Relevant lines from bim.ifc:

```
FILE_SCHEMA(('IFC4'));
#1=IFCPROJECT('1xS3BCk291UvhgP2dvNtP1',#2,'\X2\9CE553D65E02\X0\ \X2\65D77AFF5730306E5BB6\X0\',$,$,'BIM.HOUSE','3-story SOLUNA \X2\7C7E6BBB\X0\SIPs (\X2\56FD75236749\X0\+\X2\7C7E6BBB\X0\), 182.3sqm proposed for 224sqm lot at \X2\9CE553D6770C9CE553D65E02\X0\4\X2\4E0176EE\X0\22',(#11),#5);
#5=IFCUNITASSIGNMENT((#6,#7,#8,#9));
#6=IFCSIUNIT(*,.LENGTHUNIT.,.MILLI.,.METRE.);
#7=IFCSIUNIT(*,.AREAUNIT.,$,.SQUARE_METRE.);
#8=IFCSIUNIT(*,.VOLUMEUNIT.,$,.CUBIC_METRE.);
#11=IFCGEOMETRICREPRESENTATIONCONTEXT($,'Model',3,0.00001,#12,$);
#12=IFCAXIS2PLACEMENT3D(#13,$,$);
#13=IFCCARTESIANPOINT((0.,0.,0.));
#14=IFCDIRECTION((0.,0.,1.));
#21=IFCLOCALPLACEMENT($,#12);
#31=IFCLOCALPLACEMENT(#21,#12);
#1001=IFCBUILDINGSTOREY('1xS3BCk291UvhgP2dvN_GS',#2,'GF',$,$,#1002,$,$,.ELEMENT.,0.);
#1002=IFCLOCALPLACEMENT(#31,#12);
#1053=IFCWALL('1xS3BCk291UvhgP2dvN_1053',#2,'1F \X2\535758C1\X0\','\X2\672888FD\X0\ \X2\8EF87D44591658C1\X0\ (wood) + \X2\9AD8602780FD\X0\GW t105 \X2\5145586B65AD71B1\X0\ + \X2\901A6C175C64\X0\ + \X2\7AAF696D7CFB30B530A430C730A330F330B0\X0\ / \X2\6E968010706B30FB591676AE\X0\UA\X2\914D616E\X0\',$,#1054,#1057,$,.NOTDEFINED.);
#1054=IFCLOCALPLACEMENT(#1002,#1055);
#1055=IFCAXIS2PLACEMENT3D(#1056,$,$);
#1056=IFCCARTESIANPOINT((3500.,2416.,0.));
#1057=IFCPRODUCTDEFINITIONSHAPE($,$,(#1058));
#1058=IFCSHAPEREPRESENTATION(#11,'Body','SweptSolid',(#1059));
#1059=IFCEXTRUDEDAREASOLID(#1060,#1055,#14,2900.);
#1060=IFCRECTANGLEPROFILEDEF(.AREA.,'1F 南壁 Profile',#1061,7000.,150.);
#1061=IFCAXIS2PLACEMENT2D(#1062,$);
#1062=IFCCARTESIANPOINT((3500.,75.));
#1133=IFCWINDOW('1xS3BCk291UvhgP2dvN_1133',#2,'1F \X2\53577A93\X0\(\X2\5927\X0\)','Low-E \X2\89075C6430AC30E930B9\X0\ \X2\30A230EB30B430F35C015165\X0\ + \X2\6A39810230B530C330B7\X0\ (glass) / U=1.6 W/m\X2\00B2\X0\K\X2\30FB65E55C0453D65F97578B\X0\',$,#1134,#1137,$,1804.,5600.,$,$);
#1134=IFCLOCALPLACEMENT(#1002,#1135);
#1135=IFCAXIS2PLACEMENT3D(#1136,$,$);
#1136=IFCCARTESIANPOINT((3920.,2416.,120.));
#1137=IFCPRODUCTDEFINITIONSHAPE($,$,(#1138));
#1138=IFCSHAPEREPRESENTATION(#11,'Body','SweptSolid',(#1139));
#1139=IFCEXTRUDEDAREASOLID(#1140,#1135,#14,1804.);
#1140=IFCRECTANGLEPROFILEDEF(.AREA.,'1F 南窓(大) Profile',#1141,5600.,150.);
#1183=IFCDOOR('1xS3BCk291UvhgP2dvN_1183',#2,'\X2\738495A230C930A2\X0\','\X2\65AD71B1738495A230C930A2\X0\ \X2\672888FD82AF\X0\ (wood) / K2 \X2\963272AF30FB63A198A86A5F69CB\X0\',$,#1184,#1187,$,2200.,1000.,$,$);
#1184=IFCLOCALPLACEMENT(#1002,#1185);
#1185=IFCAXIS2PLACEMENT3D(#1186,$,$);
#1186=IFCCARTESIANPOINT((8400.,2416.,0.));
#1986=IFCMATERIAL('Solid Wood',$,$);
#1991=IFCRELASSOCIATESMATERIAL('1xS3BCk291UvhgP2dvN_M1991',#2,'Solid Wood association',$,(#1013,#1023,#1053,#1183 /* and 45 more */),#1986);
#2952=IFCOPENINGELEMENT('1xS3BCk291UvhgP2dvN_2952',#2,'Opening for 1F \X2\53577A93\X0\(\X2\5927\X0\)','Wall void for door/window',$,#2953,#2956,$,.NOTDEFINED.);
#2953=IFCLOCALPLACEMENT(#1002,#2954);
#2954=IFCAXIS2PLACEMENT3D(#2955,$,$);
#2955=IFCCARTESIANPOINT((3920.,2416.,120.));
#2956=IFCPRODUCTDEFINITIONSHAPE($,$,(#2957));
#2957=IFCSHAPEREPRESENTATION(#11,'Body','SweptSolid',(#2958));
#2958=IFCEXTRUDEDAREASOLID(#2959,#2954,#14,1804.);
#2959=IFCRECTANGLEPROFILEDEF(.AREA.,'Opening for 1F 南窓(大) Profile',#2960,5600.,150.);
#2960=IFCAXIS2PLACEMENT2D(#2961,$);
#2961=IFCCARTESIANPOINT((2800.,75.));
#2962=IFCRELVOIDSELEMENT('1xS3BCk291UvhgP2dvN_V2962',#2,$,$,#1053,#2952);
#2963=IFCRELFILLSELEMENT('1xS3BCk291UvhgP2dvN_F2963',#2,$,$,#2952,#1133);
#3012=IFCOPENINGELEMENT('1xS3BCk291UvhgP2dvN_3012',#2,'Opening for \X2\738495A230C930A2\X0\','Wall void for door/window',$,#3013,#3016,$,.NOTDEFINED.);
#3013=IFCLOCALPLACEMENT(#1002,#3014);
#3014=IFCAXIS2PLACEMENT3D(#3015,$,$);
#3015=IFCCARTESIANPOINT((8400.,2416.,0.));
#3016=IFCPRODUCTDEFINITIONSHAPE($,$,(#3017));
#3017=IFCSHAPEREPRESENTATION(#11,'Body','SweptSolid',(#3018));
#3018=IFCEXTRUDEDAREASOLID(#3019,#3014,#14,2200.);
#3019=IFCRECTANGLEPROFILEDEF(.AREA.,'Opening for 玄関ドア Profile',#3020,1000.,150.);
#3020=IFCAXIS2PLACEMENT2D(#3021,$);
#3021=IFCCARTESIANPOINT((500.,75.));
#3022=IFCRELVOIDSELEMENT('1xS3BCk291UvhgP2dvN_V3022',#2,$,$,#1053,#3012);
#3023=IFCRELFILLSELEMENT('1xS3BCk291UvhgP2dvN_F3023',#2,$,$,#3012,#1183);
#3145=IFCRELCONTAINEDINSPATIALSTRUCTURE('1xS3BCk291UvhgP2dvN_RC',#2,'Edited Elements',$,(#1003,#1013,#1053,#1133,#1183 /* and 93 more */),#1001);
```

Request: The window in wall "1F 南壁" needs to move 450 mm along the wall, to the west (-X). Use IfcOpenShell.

```python
import ifcopenshell
import ifcopenshell.api.geometry
import ifcopenshell.util.placement

model = ifcopenshell.open("bim.ifc")

window = model.by_guid("1xS3BCk291UvhgP2dvN_1133")
opening = window.FillsVoids[0].RelatingOpeningElement
wall = opening.VoidsElements[0].RelatingBuildingElement

wall_matrix = ifcopenshell.util.placement.get_local_placement(wall.ObjectPlacement)
shift = wall_matrix[:3, 0] * -450.0
before = ifcopenshell.util.placement.get_local_placement(window.ObjectPlacement)[:3, 3].copy()

# The window is not placed relative to its opening, so move both.
for product in (opening, window):
    matrix = ifcopenshell.util.placement.get_local_placement(product.ObjectPlacement)
    matrix[:3, 3] += shift
    ifcopenshell.api.geometry.edit_object_placement(model, product=product, matrix=matrix, is_si=False)

after = ifcopenshell.util.placement.get_local_placement(window.ObjectPlacement)[:3, 3]
print("window moved by", (after - before).round(3) + 0.0)

model.write("bim_v2.ifc")
```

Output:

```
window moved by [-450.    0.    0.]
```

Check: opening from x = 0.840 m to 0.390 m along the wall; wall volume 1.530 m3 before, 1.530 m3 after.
